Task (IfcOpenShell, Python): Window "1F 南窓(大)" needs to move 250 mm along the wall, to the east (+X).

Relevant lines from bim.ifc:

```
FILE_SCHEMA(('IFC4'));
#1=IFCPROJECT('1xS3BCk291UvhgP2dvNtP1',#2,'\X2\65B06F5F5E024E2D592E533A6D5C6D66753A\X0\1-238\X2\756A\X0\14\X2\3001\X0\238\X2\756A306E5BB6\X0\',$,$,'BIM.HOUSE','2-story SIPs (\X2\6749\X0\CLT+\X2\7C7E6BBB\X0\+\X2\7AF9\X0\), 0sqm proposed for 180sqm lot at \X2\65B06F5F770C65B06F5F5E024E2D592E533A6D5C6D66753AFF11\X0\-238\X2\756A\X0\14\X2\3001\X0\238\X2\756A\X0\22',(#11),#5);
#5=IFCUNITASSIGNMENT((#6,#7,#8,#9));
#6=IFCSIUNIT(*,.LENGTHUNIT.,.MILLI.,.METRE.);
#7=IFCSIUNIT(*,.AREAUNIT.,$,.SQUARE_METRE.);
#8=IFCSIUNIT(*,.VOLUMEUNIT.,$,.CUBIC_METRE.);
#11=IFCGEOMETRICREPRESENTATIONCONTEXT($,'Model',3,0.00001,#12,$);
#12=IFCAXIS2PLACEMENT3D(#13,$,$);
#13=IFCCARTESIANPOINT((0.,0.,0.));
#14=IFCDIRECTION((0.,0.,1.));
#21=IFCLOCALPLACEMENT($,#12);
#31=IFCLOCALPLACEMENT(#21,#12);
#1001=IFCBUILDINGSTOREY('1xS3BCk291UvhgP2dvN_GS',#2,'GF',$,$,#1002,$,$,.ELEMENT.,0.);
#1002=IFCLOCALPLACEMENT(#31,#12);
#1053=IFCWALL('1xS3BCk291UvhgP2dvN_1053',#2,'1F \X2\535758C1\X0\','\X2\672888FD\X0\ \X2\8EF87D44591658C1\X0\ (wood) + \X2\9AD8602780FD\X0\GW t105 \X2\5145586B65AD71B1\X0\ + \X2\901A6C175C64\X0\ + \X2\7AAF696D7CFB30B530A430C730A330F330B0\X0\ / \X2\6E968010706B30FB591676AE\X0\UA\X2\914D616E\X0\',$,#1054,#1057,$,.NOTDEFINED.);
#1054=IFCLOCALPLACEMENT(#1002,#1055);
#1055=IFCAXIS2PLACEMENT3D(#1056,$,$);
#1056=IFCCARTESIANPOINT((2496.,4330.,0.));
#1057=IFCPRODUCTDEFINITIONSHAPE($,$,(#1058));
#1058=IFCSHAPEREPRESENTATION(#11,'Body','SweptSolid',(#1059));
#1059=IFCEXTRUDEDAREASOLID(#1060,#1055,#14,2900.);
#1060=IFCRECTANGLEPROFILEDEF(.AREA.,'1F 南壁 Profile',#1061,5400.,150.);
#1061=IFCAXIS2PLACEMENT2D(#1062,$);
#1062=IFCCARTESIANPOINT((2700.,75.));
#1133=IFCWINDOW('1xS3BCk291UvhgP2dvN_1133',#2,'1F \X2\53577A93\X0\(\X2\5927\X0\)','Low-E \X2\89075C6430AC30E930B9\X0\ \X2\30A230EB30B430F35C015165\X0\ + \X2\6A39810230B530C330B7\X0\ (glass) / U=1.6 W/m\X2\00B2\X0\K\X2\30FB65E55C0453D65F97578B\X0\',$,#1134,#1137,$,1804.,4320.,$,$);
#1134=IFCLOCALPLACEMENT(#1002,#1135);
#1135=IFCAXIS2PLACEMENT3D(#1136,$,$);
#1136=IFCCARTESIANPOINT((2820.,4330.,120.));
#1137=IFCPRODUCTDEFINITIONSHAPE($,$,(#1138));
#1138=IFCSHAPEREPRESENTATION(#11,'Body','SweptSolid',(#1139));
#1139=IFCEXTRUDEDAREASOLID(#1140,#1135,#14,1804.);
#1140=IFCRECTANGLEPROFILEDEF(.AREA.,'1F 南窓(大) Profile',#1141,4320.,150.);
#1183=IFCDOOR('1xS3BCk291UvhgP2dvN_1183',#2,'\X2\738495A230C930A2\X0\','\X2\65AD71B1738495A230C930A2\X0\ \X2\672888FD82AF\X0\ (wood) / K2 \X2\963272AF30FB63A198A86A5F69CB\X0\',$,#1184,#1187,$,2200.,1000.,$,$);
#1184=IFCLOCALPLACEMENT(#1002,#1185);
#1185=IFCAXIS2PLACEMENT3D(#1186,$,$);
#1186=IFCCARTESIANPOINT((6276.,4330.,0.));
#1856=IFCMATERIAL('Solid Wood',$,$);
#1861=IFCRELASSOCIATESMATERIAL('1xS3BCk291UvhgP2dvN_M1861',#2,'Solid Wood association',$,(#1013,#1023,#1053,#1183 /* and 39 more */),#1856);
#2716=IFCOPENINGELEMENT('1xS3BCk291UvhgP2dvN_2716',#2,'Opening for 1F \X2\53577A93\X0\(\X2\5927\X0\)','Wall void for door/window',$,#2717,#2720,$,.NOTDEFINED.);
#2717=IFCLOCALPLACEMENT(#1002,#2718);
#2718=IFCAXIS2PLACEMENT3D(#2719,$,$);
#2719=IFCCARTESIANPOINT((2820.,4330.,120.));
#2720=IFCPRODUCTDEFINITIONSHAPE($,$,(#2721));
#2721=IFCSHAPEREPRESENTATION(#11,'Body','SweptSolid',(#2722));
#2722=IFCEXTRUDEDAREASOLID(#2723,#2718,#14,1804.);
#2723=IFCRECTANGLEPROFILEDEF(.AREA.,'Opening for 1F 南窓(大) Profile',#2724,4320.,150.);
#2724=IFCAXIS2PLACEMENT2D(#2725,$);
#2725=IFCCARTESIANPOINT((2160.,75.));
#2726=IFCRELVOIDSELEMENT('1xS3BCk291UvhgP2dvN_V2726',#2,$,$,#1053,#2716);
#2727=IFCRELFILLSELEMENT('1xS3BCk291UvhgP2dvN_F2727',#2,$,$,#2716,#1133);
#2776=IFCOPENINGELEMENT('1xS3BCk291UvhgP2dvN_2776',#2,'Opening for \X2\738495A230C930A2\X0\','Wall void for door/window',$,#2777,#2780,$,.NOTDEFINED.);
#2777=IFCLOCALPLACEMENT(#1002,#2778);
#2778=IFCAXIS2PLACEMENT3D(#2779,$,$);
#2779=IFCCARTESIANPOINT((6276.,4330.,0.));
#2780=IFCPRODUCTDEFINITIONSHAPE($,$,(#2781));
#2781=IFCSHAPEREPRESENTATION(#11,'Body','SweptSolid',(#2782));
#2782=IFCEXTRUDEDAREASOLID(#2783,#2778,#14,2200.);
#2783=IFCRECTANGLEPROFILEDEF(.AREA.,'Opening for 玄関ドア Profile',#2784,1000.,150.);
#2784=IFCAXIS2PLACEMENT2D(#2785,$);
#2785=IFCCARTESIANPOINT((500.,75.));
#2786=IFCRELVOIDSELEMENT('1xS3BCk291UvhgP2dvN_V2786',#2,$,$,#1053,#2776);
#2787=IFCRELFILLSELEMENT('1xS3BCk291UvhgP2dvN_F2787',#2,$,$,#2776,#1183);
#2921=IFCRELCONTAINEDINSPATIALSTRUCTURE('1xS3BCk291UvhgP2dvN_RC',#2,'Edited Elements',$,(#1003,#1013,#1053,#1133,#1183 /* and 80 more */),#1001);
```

```python
import ifcopenshell
import ifcopenshell.api.geometry
import ifcopenshell.util.placement
import ifcopenshell.util.unit

model = ifcopenshell.open("bim.ifc")
unit_scale = ifcopenshell.util.unit.calculate_unit_scale(model)

window = model.by_guid("1xS3BCk291UvhgP2dvN_1133")
opening = window.FillsVoids[0].RelatingOpeningElement
wall = opening.VoidsElements[0].RelatingBuildingElement

wall_matrix = ifcopenshell.util.placement.get_local_placement(wall.ObjectPlacement)
shift = wall_matrix[:3, 0] * 0.25 / unit_scale
before = ifcopenshell.util.placement.get_local_placement(window.ObjectPlacement)[:3, 3].copy()

# The window is not placed relative to its opening, so move both.
for product in (opening, window):
    matrix = ifcopenshell.util.placement.get_local_placement(product.ObjectPlacement)
    matrix[:3, 3] += shift
    ifcopenshell.api.geometry.edit_object_placement(model, product=product, matrix=matrix, is_si=False)

after = ifcopenshell.util.placement.get_local_placement(window.ObjectPlacement)[:3, 3]
print("window moved by", (after - before).round(3) + 0.0)

model.write("bim_v2.ifc")
```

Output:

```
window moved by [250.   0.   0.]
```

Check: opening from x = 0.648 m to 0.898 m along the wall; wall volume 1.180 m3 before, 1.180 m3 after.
